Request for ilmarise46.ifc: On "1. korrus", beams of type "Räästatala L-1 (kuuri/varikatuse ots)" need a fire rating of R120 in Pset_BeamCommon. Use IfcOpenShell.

First a look at what the model holds.

```python
import ifcopenshell
import ifcopenshell.util.element

model = ifcopenshell.open("ilmarise46.ifc")
print(model.schema)
storey = next(s for s in model.by_type("IfcBuildingStorey") if s.Name == "1. korrus")
beams = [e for e in ifcopenshell.util.element.get_decomposition(storey) if e.is_a("IfcBeam")]
seen = {}
for e in beams:
    element_type = ifcopenshell.util.element.get_type(e)
    key = (element_type.Name if element_type != e and element_type else None, ifcopenshell.util.element.get_pset(e, "Pset_BeamCommon", "FireRating"))
    seen[key] = seen.get(key, 0) + 1
for (name, value), count in sorted(seen.items(), key=str):
    print(count, "x", name, "|", value)
```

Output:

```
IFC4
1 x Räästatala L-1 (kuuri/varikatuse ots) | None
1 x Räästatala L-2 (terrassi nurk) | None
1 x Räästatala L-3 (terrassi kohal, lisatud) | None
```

```python
import ifcopenshell
import ifcopenshell.api.pset
import ifcopenshell.util.element

model = ifcopenshell.open("ilmarise46.ifc")

storey = next(s for s in model.by_type("IfcBuildingStorey") if s.Name == "1. korrus")
beams = [e for e in ifcopenshell.util.element.get_decomposition(storey) if e.is_a("IfcBeam")]

count = 0
for e in beams:
    element_type = ifcopenshell.util.element.get_type(e)
    if element_type in (None, e) or element_type.Name != "Räästatala L-1 (kuuri/varikatuse ots)":
        continue
    # add_pset returns the element's existing set when there is one.
    pset = ifcopenshell.api.pset.add_pset(model, product=e, name="Pset_BeamCommon")
    ifcopenshell.api.pset.edit_pset(model, pset=pset, properties={"FireRating": "R120"})
    count += 1

print(count, "beams updated")

model.write("ilmarise46_edited.ifc")
```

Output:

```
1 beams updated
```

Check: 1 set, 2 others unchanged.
